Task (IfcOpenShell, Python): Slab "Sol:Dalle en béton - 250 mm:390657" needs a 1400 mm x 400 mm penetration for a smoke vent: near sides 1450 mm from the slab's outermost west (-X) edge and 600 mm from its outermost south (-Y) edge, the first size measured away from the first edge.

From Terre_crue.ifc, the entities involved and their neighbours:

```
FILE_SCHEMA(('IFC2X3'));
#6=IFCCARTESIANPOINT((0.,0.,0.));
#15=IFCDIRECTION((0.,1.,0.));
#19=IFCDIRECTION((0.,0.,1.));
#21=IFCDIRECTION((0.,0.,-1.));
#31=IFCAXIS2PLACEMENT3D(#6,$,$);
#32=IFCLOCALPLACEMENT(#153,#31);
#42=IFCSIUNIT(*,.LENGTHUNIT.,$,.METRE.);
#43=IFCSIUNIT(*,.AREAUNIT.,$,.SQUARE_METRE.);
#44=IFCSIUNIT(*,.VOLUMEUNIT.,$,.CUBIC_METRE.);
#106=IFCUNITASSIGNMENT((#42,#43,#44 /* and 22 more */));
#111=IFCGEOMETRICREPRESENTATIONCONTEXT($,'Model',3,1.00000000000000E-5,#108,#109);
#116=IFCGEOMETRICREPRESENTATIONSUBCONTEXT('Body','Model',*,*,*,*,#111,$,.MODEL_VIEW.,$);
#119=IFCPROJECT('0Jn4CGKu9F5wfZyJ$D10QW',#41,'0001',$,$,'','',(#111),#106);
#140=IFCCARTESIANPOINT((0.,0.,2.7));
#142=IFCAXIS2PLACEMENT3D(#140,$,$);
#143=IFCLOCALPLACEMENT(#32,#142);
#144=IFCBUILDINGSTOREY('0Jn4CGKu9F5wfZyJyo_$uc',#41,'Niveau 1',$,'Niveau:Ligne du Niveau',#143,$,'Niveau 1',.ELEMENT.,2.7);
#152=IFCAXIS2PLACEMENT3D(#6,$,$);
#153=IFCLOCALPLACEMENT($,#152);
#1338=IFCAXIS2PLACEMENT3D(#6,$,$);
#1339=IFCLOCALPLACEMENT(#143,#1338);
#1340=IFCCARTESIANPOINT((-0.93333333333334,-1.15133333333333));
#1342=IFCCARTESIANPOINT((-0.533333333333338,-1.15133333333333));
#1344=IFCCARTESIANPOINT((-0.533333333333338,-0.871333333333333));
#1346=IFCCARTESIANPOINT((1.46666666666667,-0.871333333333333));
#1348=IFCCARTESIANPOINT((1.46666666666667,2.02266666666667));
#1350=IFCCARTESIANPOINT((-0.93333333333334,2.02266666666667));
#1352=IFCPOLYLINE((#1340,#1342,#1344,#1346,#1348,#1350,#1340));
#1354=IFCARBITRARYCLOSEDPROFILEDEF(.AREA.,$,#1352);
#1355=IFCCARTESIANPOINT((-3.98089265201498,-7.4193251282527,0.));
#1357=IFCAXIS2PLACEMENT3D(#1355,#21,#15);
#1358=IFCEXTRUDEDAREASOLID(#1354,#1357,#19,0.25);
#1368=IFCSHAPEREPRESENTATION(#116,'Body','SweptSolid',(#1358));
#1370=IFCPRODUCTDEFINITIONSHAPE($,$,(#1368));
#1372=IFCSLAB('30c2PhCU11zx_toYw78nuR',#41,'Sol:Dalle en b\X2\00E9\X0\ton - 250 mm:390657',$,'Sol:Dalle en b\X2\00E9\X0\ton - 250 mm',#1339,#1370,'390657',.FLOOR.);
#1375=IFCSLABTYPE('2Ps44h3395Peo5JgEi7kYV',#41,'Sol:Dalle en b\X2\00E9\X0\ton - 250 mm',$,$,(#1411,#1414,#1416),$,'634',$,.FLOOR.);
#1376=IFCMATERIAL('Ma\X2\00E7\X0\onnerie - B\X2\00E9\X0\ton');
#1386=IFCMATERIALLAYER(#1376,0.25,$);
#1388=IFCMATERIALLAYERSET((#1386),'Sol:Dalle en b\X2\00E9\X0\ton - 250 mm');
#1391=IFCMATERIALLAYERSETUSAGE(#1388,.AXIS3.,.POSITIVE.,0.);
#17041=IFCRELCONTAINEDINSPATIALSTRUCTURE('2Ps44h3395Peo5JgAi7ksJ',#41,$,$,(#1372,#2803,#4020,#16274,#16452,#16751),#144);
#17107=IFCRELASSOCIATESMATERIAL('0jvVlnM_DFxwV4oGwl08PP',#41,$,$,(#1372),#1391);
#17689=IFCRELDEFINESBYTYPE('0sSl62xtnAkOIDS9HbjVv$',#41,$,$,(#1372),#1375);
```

```python
import numpy as np
import ifcopenshell
import ifcopenshell.api.feature
import ifcopenshell.api.geometry
import ifcopenshell.api.root
import ifcopenshell.geom
import ifcopenshell.util.placement
import ifcopenshell.util.representation
import ifcopenshell.util.shape
import ifcopenshell.util.unit

model = ifcopenshell.open("Terre_crue.ifc")
unit_scale = ifcopenshell.util.unit.calculate_unit_scale(model)
settings = ifcopenshell.geom.settings()


def volume(element):
    """Net volume in cubic metres, openings subtracted."""
    shape = ifcopenshell.geom.create_shape(settings, element)
    return ifcopenshell.util.shape.get_volume(shape.geometry)


slab = model.by_guid("30c2PhCU11zx_toYw78nuR")
before = volume(slab)

# Extent in the slab's own axes, in metres. The edges named are its -X and -Y sides.
slab_shape = ifcopenshell.geom.create_shape(settings, slab)
vertices = ifcopenshell.util.shape.get_vertices(slab_shape.geometry)
x_min, y_min, bottom = vertices.min(axis=0)
top = vertices[:, 2].max()

opening = ifcopenshell.api.root.create_entity(model, ifc_class="IfcOpeningElement", name="Smoke vent opening")
context = ifcopenshell.util.representation.get_context(model, "Model", "Body", "MODEL_VIEW")
width, depth = 1.4, 0.4
outline = [(0.0, 0.0), (width, 0.0), (width, depth), (0.0, depth), (0.0, 0.0)]
# Overshoot both faces by 50 mm so the cut is clean.
shape = ifcopenshell.api.geometry.add_slab_representation(
    model, context=context, depth=top - bottom + 0.1, polyline=outline
)
ifcopenshell.api.geometry.assign_representation(model, product=opening, representation=shape)

matrix = ifcopenshell.util.placement.get_local_placement(slab.ObjectPlacement)
matrix[:, 3] = matrix @ np.append(np.array([x_min + 1.45, y_min + 0.6, bottom - 0.05]) / unit_scale, 1.0)
ifcopenshell.api.geometry.edit_object_placement(model, product=opening, matrix=matrix, is_si=False)
ifcopenshell.api.feature.add_feature(model, feature=opening, element=slab)

after = volume(slab)

print(f"slab volume {before:.3f} -> {after:.3f} m3")

model.write("Terre_crue-out.ifc")
```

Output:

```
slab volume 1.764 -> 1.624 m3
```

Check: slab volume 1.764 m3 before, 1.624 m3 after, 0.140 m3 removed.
